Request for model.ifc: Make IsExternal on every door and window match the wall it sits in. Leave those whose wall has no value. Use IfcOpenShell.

First a look at what the model holds.

```python
import ifcopenshell
import ifcopenshell.util.element

model = ifcopenshell.open("model.ifc")
print(model.schema)
seen = {}
for e in model.by_type("IfcDoor") + model.by_type("IfcWindow"):
    if not e.FillsVoids:
        continue
    host = e.FillsVoids[0].RelatingOpeningElement.VoidsElements[0].RelatingBuildingElement
    own = ifcopenshell.util.element.get_pset(e, f"Pset_{e.is_a()[3:].removesuffix('StandardCase')}Common", "IsExternal")
    wall = ifcopenshell.util.element.get_pset(host, "Pset_WallCommon", "IsExternal")
    seen[e.is_a(), own, wall] = seen.get((e.is_a(), own, wall), 0) + 1
for (cls, own, wall), count in sorted(seen.items(), key=str):
    print(count, cls, "IsExternal:", own, "| host wall:", wall)
```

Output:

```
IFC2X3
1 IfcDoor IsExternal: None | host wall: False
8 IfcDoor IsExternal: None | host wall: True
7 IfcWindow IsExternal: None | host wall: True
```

```python
import ifcopenshell
import ifcopenshell.api.pset
import ifcopenshell.util.element

model = ifcopenshell.open("model.ifc")

count = 0
for ifc_class, pset_name in (("IfcDoor", "Pset_DoorCommon"), ("IfcWindow", "Pset_WindowCommon")):
    for e in model.by_type(ifc_class):
        if not e.FillsVoids:
            continue
        host = e.FillsVoids[0].RelatingOpeningElement.VoidsElements[0].RelatingBuildingElement
        external = ifcopenshell.util.element.get_pset(host, "Pset_WallCommon", "IsExternal")
        if external is None or ifcopenshell.util.element.get_pset(e, pset_name, "IsExternal") == external:
            continue
        pset = ifcopenshell.api.pset.add_pset(model, product=e, name=pset_name)
        ifcopenshell.api.pset.edit_pset(model, pset=pset, properties={"IsExternal": external})
        count += 1

print(count, "updated")

model.write("model_edited.ifc")
```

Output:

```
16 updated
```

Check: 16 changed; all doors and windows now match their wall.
